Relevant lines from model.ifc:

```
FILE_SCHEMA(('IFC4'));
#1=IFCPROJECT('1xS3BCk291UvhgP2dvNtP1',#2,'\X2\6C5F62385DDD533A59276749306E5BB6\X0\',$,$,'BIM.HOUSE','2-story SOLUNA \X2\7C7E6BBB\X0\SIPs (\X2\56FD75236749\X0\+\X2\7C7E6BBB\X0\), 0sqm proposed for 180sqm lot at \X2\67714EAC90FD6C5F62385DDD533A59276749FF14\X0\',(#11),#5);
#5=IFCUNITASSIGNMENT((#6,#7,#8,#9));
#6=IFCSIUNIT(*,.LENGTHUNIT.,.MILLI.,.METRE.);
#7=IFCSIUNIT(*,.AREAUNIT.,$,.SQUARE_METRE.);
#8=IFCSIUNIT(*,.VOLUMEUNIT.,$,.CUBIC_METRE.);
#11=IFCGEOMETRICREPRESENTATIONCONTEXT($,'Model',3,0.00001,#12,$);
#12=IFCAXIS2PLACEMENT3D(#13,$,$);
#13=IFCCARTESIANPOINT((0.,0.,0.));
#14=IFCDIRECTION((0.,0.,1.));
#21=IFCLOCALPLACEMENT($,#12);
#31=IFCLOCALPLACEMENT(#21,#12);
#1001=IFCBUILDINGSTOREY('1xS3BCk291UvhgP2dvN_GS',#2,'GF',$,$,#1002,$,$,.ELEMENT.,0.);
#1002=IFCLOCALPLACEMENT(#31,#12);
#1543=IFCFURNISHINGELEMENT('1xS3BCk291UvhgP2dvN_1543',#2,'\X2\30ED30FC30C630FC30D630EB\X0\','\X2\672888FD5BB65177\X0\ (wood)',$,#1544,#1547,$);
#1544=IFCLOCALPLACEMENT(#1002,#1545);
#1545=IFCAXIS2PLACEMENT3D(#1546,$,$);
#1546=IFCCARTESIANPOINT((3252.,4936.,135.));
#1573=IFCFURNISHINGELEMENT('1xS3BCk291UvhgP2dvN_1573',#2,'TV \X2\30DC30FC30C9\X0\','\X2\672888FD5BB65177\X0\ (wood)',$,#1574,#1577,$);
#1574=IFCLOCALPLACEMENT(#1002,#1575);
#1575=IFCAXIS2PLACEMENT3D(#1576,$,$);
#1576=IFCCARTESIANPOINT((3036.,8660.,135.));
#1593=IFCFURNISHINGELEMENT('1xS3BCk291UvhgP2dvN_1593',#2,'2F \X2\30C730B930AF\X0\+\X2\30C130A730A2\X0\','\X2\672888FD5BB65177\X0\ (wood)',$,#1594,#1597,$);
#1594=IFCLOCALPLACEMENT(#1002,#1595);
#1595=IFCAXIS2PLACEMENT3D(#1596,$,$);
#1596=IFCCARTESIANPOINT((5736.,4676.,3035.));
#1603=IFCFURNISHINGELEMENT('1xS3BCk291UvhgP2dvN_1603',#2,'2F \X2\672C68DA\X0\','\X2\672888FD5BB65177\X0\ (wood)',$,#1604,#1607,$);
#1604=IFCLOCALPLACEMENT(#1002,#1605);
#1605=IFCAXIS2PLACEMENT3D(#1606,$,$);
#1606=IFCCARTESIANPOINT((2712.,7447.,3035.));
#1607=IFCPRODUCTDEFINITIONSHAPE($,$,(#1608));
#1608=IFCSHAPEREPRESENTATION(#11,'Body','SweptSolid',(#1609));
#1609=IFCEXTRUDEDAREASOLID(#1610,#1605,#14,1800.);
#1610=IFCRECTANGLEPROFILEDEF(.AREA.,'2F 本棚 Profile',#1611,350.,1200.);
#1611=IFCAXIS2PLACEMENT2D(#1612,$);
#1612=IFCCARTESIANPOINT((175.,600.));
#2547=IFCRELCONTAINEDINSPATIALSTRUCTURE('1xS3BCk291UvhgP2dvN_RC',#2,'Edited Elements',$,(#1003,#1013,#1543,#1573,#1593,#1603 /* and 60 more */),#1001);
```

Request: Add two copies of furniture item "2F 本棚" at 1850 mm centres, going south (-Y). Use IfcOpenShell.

```python
import numpy as np
import ifcopenshell
import ifcopenshell.api.geometry
import ifcopenshell.api.root
import ifcopenshell.util.element
import ifcopenshell.util.placement
import ifcopenshell.util.unit

model = ifcopenshell.open("model.ifc")
unit_scale = ifcopenshell.util.unit.calculate_unit_scale(model)


def reuse_history(source, copy):
    """copy_class also copies each property set's owner history, people and application; keep the originals."""
    for rel in copy.IsDefinedBy:
        if rel.is_a("IfcRelDefinesByProperties") and (history := rel.RelatingPropertyDefinition.OwnerHistory):
            rel.RelatingPropertyDefinition.OwnerHistory = source.OwnerHistory
            ifcopenshell.util.element.remove_deep2(model, history)


source = model.by_guid("1xS3BCk291UvhgP2dvN_1603")
base = ifcopenshell.util.placement.get_local_placement(source.ObjectPlacement)
step = np.array([0.0, -1.0, 0.0]) * 1.85 / unit_scale

for i in range(1, 3):
    copy = ifcopenshell.api.root.copy_class(model, product=source)
    copy.Representation = ifcopenshell.util.element.copy_deep(
        model, source.Representation, exclude=["IfcGeometricRepresentationContext", "IfcRepresentationMap"]
    )
    reuse_history(source, copy)
    matrix = base.copy()
    matrix[:3, 3] += i * step
    print("added at", matrix[:3, 3].round(3) + 0.0)
    ifcopenshell.api.geometry.edit_object_placement(model, product=copy, matrix=matrix, is_si=False)

model.write("model-out.ifc")
```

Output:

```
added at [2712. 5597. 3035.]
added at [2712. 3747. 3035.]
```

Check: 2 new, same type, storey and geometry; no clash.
